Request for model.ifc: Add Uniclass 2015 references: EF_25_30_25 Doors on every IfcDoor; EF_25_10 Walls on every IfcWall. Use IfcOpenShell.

First a look at what the model holds.

```python
import ifcopenshell

model = ifcopenshell.open("model.ifc")
print(model.schema)
print("classifications:", [c.Name for c in model.by_type("IfcClassification")])
for ifc_class in ("IfcDoor", "IfcRoof", "IfcStair", "IfcWall", "IfcWindow"):
    print(ifc_class, len(model.by_type(ifc_class)))
```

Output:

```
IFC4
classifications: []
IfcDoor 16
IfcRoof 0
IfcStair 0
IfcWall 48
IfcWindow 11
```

```python
import ifcopenshell
import ifcopenshell.api.classification

model = ifcopenshell.open("model.ifc")

system = ifcopenshell.api.classification.add_classification(model, classification="Uniclass 2015")

codes = {
    "IfcDoor": ("EF_25_30_25", "Doors"),
    "IfcWall": ("EF_25_10", "Walls"),
}
for ifc_class, (code, name) in codes.items():
    products = model.by_type(ifc_class)
    ifcopenshell.api.classification.add_reference(
        model, products=products, classification=system, identification=code, name=name
    )
    print(code, len(products))

model.write("model_updated.ifc")
```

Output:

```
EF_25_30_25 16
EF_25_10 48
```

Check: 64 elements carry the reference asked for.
